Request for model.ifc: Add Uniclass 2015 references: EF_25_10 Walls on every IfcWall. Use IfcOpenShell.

First a look at what the model holds.

```python
import ifcopenshell

model = ifcopenshell.open("model.ifc")
print(model.schema)
print("classifications:", [c.Name for c in model.by_type("IfcClassification")])
for ifc_class in ("IfcDoor", "IfcRoof", "IfcStair", "IfcWall", "IfcWindow"):
    print(ifc_class, len(model.by_type(ifc_class)))
```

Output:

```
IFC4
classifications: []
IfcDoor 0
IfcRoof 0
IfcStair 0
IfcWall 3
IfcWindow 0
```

```python
import ifcopenshell
import ifcopenshell.api.classification

model = ifcopenshell.open("model.ifc")

system = ifcopenshell.api.classification.add_classification(model, classification="Uniclass 2015")

codes = {
    "IfcWall": ("EF_25_10", "Walls"),
}
for ifc_class, (code, name) in codes.items():
    products = model.by_type(ifc_class)
    ifcopenshell.api.classification.add_reference(
        model, products=products, classification=system, identification=code, name=name
    )
    print(code, len(products))

model.write("model_v2.ifc")
```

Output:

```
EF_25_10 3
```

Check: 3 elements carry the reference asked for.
